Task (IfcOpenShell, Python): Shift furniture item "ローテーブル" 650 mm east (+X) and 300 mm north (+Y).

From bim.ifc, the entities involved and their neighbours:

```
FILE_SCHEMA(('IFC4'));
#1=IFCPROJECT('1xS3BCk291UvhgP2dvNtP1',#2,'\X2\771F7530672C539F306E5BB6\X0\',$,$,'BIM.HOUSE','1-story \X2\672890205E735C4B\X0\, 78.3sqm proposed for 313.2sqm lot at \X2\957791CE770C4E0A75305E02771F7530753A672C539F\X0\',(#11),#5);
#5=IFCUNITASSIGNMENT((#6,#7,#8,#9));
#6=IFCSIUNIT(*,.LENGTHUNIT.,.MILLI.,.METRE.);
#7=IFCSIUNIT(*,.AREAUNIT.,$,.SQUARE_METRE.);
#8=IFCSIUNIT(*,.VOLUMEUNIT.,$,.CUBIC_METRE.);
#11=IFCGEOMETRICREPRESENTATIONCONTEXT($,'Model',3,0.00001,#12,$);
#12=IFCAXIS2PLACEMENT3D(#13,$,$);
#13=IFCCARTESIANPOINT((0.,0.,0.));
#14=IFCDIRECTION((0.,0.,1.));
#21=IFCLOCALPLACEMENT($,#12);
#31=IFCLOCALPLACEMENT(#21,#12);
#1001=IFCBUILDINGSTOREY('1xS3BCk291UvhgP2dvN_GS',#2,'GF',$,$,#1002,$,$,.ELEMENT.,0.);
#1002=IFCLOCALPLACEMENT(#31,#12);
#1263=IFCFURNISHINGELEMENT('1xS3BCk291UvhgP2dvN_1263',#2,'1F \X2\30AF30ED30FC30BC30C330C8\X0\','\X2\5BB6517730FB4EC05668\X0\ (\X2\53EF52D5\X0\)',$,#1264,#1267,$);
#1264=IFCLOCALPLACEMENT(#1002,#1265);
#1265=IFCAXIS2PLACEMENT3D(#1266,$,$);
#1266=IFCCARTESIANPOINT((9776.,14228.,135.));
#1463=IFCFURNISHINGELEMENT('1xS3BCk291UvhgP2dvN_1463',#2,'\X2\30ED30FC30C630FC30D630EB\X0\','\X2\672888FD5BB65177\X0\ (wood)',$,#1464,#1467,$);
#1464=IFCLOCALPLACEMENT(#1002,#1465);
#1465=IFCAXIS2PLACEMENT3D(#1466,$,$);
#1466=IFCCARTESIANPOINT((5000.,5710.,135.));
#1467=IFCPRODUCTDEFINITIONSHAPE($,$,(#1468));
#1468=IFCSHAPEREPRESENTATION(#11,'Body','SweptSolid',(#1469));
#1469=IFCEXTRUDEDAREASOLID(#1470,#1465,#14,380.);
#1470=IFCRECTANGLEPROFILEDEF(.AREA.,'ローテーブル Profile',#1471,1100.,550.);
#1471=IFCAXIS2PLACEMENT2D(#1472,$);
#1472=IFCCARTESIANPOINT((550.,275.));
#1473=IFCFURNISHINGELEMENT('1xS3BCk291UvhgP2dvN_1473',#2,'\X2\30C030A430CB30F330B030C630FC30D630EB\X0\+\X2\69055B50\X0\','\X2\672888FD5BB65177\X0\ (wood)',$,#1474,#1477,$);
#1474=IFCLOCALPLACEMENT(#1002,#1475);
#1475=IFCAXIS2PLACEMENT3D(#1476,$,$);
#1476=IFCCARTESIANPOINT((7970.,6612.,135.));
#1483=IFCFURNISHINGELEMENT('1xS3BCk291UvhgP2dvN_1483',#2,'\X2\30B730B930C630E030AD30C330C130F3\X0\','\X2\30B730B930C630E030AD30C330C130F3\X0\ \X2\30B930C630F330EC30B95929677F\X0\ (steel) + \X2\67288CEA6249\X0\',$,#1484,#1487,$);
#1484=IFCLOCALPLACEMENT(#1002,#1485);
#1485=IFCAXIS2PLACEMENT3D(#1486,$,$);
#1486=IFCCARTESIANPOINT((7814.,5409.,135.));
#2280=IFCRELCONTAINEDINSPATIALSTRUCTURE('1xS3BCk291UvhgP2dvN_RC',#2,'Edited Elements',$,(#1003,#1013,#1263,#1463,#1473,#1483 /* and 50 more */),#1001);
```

```python
import ifcopenshell
import ifcopenshell.api.geometry
import ifcopenshell.util.placement
import ifcopenshell.util.unit

model = ifcopenshell.open("bim.ifc")
unit_scale = ifcopenshell.util.unit.calculate_unit_scale(model)

item = model.by_guid("1xS3BCk291UvhgP2dvN_1463")
matrix = ifcopenshell.util.placement.get_local_placement(item.ObjectPlacement)
matrix[0, 3] += 0.65 / unit_scale
matrix[1, 3] += 0.3 / unit_scale
ifcopenshell.api.geometry.edit_object_placement(model, product=item, matrix=matrix, is_si=False)

print(ifcopenshell.util.placement.get_local_placement(item.ObjectPlacement).round(3) + 0.0)

model.write("bim_edited.ifc")
```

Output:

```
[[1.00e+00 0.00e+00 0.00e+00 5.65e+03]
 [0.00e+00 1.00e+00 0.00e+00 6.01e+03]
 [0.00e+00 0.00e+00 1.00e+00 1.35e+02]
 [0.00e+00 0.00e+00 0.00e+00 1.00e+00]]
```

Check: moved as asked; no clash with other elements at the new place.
